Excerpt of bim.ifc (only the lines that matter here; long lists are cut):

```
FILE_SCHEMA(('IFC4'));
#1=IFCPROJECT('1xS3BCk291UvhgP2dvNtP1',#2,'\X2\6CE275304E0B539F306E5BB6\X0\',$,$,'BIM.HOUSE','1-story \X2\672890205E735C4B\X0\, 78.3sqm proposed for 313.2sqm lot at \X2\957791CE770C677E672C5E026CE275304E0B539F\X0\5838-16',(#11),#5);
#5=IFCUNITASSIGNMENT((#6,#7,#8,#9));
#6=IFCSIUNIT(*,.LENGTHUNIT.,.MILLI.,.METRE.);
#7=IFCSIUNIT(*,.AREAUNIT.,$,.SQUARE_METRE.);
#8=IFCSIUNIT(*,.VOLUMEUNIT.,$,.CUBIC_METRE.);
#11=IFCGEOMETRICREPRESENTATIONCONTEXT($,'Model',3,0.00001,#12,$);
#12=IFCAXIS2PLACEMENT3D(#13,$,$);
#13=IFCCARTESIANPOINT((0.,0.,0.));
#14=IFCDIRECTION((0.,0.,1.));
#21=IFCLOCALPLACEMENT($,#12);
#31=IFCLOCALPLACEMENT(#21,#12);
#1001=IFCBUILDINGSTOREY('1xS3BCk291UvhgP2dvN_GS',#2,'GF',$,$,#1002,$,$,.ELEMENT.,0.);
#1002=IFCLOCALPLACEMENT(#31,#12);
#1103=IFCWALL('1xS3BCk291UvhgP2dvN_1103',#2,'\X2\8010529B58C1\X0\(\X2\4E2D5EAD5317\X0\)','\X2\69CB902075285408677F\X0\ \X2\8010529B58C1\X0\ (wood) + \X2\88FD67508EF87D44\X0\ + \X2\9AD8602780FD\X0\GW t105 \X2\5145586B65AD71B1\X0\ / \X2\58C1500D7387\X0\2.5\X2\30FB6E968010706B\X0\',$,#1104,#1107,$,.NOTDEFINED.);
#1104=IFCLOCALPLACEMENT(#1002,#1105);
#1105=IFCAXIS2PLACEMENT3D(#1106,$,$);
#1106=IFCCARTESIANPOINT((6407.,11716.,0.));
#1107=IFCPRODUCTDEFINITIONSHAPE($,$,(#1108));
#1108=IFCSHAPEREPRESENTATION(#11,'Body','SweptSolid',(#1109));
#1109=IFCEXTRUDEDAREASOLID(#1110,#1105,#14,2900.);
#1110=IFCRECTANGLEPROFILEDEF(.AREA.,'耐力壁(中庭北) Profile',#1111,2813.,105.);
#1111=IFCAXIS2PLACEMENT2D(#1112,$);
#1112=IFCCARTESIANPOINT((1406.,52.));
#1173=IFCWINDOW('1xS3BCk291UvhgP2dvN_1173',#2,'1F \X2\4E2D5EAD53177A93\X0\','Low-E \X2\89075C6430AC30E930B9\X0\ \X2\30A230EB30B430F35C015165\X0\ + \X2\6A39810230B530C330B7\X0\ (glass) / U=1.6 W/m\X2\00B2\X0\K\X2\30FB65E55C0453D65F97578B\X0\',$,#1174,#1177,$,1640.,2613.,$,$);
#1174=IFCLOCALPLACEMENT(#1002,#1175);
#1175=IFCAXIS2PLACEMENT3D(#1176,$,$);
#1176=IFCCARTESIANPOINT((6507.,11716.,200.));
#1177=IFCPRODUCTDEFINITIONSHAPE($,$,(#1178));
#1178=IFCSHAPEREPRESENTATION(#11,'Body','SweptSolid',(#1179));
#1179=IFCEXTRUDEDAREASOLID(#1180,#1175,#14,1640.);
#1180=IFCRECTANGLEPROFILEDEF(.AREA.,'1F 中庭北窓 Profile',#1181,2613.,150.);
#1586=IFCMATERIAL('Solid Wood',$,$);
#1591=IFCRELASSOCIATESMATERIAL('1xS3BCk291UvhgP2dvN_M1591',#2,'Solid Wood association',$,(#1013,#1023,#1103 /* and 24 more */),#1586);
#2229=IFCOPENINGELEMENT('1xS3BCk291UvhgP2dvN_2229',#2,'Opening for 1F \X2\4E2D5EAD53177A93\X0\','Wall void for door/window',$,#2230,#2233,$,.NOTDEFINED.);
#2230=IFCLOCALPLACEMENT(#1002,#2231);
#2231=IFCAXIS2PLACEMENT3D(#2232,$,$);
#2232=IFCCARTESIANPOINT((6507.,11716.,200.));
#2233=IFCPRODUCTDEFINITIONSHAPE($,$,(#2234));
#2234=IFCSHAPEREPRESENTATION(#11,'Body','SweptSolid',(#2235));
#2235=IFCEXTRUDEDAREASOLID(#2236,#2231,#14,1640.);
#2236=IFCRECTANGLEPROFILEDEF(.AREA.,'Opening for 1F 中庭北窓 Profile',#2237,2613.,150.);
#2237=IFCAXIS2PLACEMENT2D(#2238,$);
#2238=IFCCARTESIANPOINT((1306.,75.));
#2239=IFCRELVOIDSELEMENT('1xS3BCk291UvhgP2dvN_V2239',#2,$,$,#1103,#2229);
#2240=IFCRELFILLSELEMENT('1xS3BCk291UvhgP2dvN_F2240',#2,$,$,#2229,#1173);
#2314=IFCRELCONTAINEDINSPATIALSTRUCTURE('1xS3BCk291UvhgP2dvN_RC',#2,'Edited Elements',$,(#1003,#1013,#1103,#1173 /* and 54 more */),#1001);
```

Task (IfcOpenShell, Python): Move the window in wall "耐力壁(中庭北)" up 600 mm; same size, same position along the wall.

```python
import numpy as np
import ifcopenshell
import ifcopenshell.api.geometry
import ifcopenshell.util.placement
import ifcopenshell.util.unit

model = ifcopenshell.open("bim.ifc")
unit_scale = ifcopenshell.util.unit.calculate_unit_scale(model)

window = model.by_guid("1xS3BCk291UvhgP2dvN_1173")
opening = window.FillsVoids[0].RelatingOpeningElement
dz = 600.0

shift = np.array([0.0, 0.0, dz])
# The window is not placed relative to its opening, so move both.
for product in (opening, window):
    matrix = ifcopenshell.util.placement.get_local_placement(product.ObjectPlacement)
    matrix[:3, 3] += shift
    ifcopenshell.api.geometry.edit_object_placement(model, product=product, matrix=matrix, is_si=False)

print(f"moved by {dz * unit_scale:+.3f} m")

model.write("bim_v2.ifc")
```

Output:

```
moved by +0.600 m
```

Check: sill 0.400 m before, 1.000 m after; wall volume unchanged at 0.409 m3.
